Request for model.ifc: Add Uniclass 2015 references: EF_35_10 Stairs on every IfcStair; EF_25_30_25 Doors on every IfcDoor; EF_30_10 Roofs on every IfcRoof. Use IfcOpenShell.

First a look at what the model holds.

```python
import ifcopenshell

model = ifcopenshell.open("model.ifc")
print(model.schema)
print("classifications:", [c.Name for c in model.by_type("IfcClassification")])
for ifc_class in ("IfcDoor", "IfcRoof", "IfcStair", "IfcWall", "IfcWindow"):
    print(ifc_class, len(model.by_type(ifc_class)))
```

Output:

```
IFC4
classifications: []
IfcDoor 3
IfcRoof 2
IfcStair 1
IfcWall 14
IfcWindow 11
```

```python
import ifcopenshell
import ifcopenshell.api.classification

model = ifcopenshell.open("model.ifc")

system = ifcopenshell.api.classification.add_classification(model, classification="Uniclass 2015")

codes = {
    "IfcStair": ("EF_35_10", "Stairs"),
    "IfcDoor": ("EF_25_30_25", "Doors"),
    "IfcRoof": ("EF_30_10", "Roofs"),
}
for ifc_class, (code, name) in codes.items():
    products = model.by_type(ifc_class)
    ifcopenshell.api.classification.add_reference(
        model, products=products, classification=system, identification=code, name=name
    )
    print(code, len(products))

model.write("model_updated.ifc")
```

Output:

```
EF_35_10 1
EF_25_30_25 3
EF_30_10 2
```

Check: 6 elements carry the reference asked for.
